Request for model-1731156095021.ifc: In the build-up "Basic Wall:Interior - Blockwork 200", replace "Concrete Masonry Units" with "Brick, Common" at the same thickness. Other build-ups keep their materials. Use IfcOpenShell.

First a look at what the model holds.

```python
import ifcopenshell
import ifcopenshell.util.element

model = ifcopenshell.open("model-1731156095021.ifc")
print(model.schema)
for layer_set in model.by_type("IfcMaterialLayerSet"):
    if layer_set.LayerSetName == "Basic Wall:Interior - Blockwork 200":
        for layer in layer_set.MaterialLayers:
            print(layer.id(), layer.Material and layer.Material.Name, layer.LayerThickness, sep=" | ")
        print(len(ifcopenshell.util.element.get_elements_by_material(model, layer_set)), "elements and types use it")
print(sorted(m.Name for m in model.by_type("IfcMaterial") if m.Name)[:60])
```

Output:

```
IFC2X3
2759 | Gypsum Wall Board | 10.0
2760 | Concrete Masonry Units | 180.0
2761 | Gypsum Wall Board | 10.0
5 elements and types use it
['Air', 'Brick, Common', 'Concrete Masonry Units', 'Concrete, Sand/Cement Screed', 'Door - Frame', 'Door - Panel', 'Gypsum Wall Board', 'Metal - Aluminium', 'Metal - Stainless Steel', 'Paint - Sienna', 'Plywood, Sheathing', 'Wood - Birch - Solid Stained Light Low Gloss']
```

```python
import ifcopenshell
import ifcopenshell.api.material

model = ifcopenshell.open("model-1731156095021.ifc")

layer_set = next(s for s in model.by_type("IfcMaterialLayerSet") if s.LayerSetName == "Basic Wall:Interior - Blockwork 200")
layer = next(l for l in layer_set.MaterialLayers if l.Material and l.Material.Name == "Concrete Masonry Units")
material = next(m for m in model.by_type("IfcMaterial") if m.Name == "Brick, Common")

# Point this one layer at the other material; renaming the old one would change it everywhere.
ifcopenshell.api.material.edit_layer(model, layer=layer, attributes={}, material=material)

print([l.Material.Name if l.Material else None for l in layer_set.MaterialLayers])

model.write("model-1731156095021_edited.ifc")
```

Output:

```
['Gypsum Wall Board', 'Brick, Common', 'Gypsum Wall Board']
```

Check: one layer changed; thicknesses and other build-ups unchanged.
